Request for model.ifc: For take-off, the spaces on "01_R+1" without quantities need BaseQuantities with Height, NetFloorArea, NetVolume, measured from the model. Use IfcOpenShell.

First a look at what the model holds.

```python
import ifcopenshell
import ifcopenshell.util.element
import ifcopenshell.util.unit

model = ifcopenshell.open("model.ifc")
print(model.schema)
for unit_type in ("LENGTHUNIT", "AREAUNIT", "VOLUMEUNIT"):
    print(unit_type, ifcopenshell.util.unit.calculate_unit_scale(model, unit_type))
storey = next(s for s in model.by_type("IfcBuildingStorey") if s.Name == "01_R+1")
spaces = [e for e in ifcopenshell.util.element.get_decomposition(storey) if e.is_a("IfcSpace")]
for e in sorted(spaces, key=lambda e: e.id()):
    print(e.id(), e.is_a(), e.Name, list(ifcopenshell.util.element.get_psets(e, qtos_only=True)), sep=" | ")
```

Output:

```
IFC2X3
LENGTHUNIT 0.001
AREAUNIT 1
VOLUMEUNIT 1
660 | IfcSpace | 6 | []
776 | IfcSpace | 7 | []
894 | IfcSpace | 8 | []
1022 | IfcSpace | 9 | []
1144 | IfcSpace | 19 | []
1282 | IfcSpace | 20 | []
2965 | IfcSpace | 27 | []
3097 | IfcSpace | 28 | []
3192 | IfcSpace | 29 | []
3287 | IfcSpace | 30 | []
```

```python
import ifcopenshell
import ifcopenshell.api.pset
import ifcopenshell.geom
import ifcopenshell.util.element
import ifcopenshell.util.shape
import ifcopenshell.util.unit

model = ifcopenshell.open("model.ifc")
unit_scale = ifcopenshell.util.unit.calculate_unit_scale(model)
area_scale = ifcopenshell.util.unit.calculate_unit_scale(model, "AREAUNIT")
volume_scale = ifcopenshell.util.unit.calculate_unit_scale(model, "VOLUMEUNIT")
settings = ifcopenshell.geom.settings()

storey = next(s for s in model.by_type("IfcBuildingStorey") if s.Name == "01_R+1")
spaces = [e for e in ifcopenshell.util.element.get_decomposition(storey) if e.is_a("IfcSpace")]

for e in sorted(spaces, key=lambda e: e.id()):
    if ifcopenshell.util.element.get_psets(e, qtos_only=True, should_inherit=False):
        continue
    # Geometry comes back in metres, in the element's own axes.
    shape = ifcopenshell.geom.create_shape(settings, e)
    values = {
        "Height": ifcopenshell.util.shape.get_z(shape.geometry) / unit_scale,
        "NetFloorArea": ifcopenshell.util.shape.get_footprint_area(shape.geometry) / area_scale,
        "NetVolume": ifcopenshell.util.shape.get_volume(shape.geometry) / volume_scale,
    }
    qto = ifcopenshell.api.pset.add_qto(model, product=e, name="BaseQuantities")
    ifcopenshell.api.pset.edit_qto(model, qto=qto, properties=values)
    print(e.id(), {k: round(v, 3) for k, v in values.items()})

model.write("model_updated.ifc")
```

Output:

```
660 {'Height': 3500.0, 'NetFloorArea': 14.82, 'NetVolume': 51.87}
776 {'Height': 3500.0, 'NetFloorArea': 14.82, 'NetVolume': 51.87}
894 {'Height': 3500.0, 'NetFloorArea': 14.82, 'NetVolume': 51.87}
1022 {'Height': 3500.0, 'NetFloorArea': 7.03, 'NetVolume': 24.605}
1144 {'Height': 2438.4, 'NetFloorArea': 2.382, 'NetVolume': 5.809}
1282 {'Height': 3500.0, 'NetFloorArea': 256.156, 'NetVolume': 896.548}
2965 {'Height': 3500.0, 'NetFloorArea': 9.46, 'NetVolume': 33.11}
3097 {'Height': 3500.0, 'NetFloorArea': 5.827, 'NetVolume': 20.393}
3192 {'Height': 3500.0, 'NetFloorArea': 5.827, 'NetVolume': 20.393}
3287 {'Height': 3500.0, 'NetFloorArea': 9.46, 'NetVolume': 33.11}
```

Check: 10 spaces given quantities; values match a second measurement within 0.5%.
